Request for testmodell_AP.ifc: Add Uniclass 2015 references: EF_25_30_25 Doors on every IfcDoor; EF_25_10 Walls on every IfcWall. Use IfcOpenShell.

First a look at what the model holds.

```python
import ifcopenshell

model = ifcopenshell.open("testmodell_AP.ifc")
print(model.schema)
print("classifications:", [c.Name for c in model.by_type("IfcClassification")])
for ifc_class in ("IfcDoor", "IfcRoof", "IfcStair", "IfcWall", "IfcWindow"):
    print(ifc_class, len(model.by_type(ifc_class)))
```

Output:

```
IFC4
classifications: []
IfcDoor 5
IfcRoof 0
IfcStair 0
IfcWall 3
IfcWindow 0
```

```python
import ifcopenshell
import ifcopenshell.api.classification

model = ifcopenshell.open("testmodell_AP.ifc")

system = ifcopenshell.api.classification.add_classification(model, classification="Uniclass 2015")

codes = {
    "IfcDoor": ("EF_25_30_25", "Doors"),
    "IfcWall": ("EF_25_10", "Walls"),
}
for ifc_class, (code, name) in codes.items():
    products = model.by_type(ifc_class)
    ifcopenshell.api.classification.add_reference(
        model, products=products, classification=system, identification=code, name=name
    )
    print(code, len(products))

model.write("testmodell_AP_rev.ifc")
```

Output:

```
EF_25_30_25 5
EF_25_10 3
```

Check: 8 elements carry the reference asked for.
